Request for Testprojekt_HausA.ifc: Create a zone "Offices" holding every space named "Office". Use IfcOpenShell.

First a look at what the model holds.

```python
import ifcopenshell

model = ifcopenshell.open("Testprojekt_HausA.ifc")
print(model.schema)
seen = {}
for space in model.by_type("IfcSpace"):
    seen[space.LongName] = seen.get(space.LongName, 0) + 1
for name, count in sorted(seen.items(), key=str):
    print(count, "x", name)
print("zones:", [z.Name for z in model.by_type("IfcZone")][:20])
```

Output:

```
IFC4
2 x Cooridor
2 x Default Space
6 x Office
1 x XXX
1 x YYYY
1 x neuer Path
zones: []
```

```python
import ifcopenshell
import ifcopenshell.api.group
import ifcopenshell.api.root

model = ifcopenshell.open("Testprojekt_HausA.ifc")

names = {"Office"}
spaces = [s for s in model.by_type("IfcSpace") if s.LongName in names]

zone = ifcopenshell.api.root.create_entity(model, ifc_class="IfcZone", name="Offices")
ifcopenshell.api.group.assign_group(model, products=spaces, group=zone)
print(len(spaces), "spaces in", zone.Name)

model.write("Testprojekt_HausA_rev.ifc")
```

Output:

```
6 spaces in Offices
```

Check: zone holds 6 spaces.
